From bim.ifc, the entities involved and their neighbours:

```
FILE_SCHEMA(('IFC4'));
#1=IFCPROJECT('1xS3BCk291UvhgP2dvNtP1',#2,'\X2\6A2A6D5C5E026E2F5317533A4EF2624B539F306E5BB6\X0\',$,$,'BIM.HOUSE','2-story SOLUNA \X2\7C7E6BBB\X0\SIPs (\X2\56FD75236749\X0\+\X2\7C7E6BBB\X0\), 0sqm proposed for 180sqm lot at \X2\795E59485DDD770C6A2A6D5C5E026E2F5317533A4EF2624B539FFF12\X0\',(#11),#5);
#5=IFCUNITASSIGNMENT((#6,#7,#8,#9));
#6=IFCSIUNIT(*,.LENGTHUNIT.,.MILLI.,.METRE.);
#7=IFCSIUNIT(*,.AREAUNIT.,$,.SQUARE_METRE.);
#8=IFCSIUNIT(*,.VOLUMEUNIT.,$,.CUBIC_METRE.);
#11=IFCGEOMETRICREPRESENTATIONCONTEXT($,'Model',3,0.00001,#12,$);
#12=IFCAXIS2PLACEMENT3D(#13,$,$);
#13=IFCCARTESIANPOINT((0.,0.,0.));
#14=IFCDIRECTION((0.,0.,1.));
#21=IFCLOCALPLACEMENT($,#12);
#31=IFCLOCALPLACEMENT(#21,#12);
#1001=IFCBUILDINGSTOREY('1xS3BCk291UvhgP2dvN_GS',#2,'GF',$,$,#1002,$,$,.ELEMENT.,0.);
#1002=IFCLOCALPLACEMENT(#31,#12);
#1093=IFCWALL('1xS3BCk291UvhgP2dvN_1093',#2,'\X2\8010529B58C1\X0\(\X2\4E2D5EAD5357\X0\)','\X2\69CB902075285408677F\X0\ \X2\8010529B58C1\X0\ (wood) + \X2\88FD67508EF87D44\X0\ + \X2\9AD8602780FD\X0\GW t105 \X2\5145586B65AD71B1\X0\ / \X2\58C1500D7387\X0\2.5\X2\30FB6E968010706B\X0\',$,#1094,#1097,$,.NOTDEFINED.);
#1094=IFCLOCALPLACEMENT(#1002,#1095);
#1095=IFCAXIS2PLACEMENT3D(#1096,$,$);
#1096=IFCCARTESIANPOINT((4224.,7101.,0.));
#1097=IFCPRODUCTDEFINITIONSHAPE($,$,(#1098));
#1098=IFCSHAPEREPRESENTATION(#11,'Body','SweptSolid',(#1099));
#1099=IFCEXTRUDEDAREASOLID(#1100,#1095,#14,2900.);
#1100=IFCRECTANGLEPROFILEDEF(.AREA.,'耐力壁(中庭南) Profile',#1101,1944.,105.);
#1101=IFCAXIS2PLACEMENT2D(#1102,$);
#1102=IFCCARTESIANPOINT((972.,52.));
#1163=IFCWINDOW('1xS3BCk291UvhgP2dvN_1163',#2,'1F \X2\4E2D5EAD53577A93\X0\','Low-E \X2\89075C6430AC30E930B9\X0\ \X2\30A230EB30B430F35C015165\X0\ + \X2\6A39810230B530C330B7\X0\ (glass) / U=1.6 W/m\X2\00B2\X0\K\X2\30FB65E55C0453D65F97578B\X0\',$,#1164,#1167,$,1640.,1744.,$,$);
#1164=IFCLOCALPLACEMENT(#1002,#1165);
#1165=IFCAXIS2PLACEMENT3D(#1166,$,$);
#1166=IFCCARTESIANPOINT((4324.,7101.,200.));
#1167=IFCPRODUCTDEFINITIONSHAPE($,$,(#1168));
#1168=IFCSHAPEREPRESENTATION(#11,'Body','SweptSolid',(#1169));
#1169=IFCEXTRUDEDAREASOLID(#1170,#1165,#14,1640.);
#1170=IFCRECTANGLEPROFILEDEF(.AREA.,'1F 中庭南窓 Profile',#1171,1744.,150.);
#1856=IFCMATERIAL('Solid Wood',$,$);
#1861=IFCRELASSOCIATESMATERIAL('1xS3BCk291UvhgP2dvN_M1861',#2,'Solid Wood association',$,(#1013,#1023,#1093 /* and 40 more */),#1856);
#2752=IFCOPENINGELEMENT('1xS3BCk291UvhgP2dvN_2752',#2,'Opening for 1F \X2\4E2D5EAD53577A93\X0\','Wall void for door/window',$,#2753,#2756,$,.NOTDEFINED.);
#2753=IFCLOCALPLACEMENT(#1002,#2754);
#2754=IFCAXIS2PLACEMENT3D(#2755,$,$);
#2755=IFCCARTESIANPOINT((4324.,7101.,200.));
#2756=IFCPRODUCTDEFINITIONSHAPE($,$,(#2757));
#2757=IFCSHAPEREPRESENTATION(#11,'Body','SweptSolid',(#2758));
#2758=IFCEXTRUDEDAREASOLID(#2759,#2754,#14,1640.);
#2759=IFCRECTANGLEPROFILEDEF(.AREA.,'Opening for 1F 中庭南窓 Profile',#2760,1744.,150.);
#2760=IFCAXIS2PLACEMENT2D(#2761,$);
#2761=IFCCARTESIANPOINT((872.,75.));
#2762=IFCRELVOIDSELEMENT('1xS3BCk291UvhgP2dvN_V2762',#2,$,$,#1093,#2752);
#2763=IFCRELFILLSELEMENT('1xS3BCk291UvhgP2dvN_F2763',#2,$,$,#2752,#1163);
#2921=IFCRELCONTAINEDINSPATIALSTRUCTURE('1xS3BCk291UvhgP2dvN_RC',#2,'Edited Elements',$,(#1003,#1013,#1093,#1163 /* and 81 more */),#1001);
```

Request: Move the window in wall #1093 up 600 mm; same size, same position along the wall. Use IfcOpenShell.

```python
import numpy as np
import ifcopenshell
import ifcopenshell.api.geometry
import ifcopenshell.util.placement
import ifcopenshell.util.unit

model = ifcopenshell.open("bim.ifc")
unit_scale = ifcopenshell.util.unit.calculate_unit_scale(model)

window = model.by_guid("1xS3BCk291UvhgP2dvN_1163")
opening = window.FillsVoids[0].RelatingOpeningElement
dz = 0.6 / unit_scale

shift = np.array([0.0, 0.0, dz])
# The window is not placed relative to its opening, so move both.
for product in (opening, window):
    matrix = ifcopenshell.util.placement.get_local_placement(product.ObjectPlacement)
    matrix[:3, 3] += shift
    ifcopenshell.api.geometry.edit_object_placement(model, product=product, matrix=matrix, is_si=False)

print(f"moved by {dz * unit_scale:+.3f} m")

model.write("bim-out.ifc")
```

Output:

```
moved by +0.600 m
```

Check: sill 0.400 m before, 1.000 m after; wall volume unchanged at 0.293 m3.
